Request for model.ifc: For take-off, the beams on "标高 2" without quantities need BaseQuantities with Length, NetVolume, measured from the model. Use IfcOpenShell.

First a look at what the model holds.

```python
import ifcopenshell
import ifcopenshell.util.element
import ifcopenshell.util.unit

model = ifcopenshell.open("model.ifc")
print(model.schema)
for unit_type in ("LENGTHUNIT", "AREAUNIT", "VOLUMEUNIT"):
    print(unit_type, ifcopenshell.util.unit.calculate_unit_scale(model, unit_type))
storey = next(s for s in model.by_type("IfcBuildingStorey") if s.Name == "标高 2")
beams = [e for e in ifcopenshell.util.element.get_decomposition(storey) if e.is_a("IfcBeam")]
for e in sorted(beams, key=lambda e: e.id()):
    print(e.id(), e.is_a(), e.Name, list(ifcopenshell.util.element.get_psets(e, qtos_only=True)), sep=" | ")
```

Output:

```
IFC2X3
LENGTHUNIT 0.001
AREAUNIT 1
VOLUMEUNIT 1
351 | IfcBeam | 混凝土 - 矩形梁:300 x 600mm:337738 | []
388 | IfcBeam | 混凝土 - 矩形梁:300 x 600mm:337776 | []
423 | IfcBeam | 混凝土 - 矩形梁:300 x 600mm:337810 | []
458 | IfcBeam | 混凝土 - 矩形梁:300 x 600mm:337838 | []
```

```python
import ifcopenshell
import ifcopenshell.api.pset
import ifcopenshell.geom
import ifcopenshell.util.element
import ifcopenshell.util.shape
import ifcopenshell.util.unit

model = ifcopenshell.open("model.ifc")
unit_scale = ifcopenshell.util.unit.calculate_unit_scale(model)
volume_scale = ifcopenshell.util.unit.calculate_unit_scale(model, "VOLUMEUNIT")
settings = ifcopenshell.geom.settings()

storey = next(s for s in model.by_type("IfcBuildingStorey") if s.Name == "标高 2")
beams = [e for e in ifcopenshell.util.element.get_decomposition(storey) if e.is_a("IfcBeam")]

for e in sorted(beams, key=lambda e: e.id()):
    if ifcopenshell.util.element.get_psets(e, qtos_only=True, should_inherit=False):
        continue
    # Geometry comes back in metres, in the element's own axes.
    shape = ifcopenshell.geom.create_shape(settings, e)
    values = {
        "Length": ifcopenshell.util.shape.get_max_xyz(shape.geometry) / unit_scale,
        "NetVolume": ifcopenshell.util.shape.get_volume(shape.geometry) / volume_scale,
    }
    qto = ifcopenshell.api.pset.add_qto(model, product=e, name="BaseQuantities")
    ifcopenshell.api.pset.edit_qto(model, qto=qto, properties=values)
    print(e.id(), {k: round(v, 3) for k, v in values.items()})

model.write("model-out.ifc")
```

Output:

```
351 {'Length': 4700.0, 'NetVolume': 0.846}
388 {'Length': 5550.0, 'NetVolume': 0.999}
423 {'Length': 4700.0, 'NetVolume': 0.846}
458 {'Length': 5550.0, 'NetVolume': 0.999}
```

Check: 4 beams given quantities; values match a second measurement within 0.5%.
